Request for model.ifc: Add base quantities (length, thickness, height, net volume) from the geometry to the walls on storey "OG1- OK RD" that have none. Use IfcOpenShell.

First a look at what the model holds.

```python
import ifcopenshell
import ifcopenshell.util.element
import ifcopenshell.util.unit

model = ifcopenshell.open("model.ifc")
print(model.schema)
for unit_type in ("LENGTHUNIT", "AREAUNIT", "VOLUMEUNIT"):
    print(unit_type, ifcopenshell.util.unit.calculate_unit_scale(model, unit_type))
storey = next(s for s in model.by_type("IfcBuildingStorey") if s.Name == "OG1- OK RD")
walls = [e for e in ifcopenshell.util.element.get_decomposition(storey) if e.is_a("IfcWall")]
for e in sorted(walls, key=lambda e: e.id()):
    print(e.id(), e.is_a(), e.Name, list(ifcopenshell.util.element.get_psets(e, qtos_only=True)), sep=" | ")
```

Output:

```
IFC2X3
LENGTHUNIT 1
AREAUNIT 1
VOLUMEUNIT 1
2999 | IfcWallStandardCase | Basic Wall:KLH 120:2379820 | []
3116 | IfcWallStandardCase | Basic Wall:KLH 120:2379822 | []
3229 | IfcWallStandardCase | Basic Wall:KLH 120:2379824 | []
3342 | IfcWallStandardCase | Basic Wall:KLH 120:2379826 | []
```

```python
import ifcopenshell
import ifcopenshell.api.pset
import ifcopenshell.geom
import ifcopenshell.util.element
import ifcopenshell.util.shape
import ifcopenshell.util.unit

model = ifcopenshell.open("model.ifc")
unit_scale = ifcopenshell.util.unit.calculate_unit_scale(model)
volume_scale = ifcopenshell.util.unit.calculate_unit_scale(model, "VOLUMEUNIT")
settings = ifcopenshell.geom.settings()

storey = next(s for s in model.by_type("IfcBuildingStorey") if s.Name == "OG1- OK RD")
walls = [e for e in ifcopenshell.util.element.get_decomposition(storey) if e.is_a("IfcWall")]

for e in sorted(walls, key=lambda e: e.id()):
    if ifcopenshell.util.element.get_psets(e, qtos_only=True, should_inherit=False):
        continue
    # Geometry comes back in metres, in the element's own axes.
    shape = ifcopenshell.geom.create_shape(settings, e)
    values = {
        "Length": ifcopenshell.util.shape.get_x(shape.geometry) / unit_scale,
        "Width": ifcopenshell.util.shape.get_y(shape.geometry) / unit_scale,
        "Height": ifcopenshell.util.shape.get_z(shape.geometry) / unit_scale,
        "NetVolume": ifcopenshell.util.shape.get_volume(shape.geometry) / volume_scale,
    }
    qto = ifcopenshell.api.pset.add_qto(model, product=e, name="BaseQuantities")
    ifcopenshell.api.pset.edit_qto(model, qto=qto, properties=values)
    print(e.id(), {k: round(v, 3) for k, v in values.items()})

model.write("model_updated.ifc")
```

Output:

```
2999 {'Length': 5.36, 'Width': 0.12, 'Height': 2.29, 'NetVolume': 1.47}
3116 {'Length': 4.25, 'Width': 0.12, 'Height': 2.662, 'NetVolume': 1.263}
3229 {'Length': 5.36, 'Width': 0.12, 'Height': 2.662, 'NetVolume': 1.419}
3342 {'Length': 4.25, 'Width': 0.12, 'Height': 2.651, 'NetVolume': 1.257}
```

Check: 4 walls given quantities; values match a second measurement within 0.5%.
